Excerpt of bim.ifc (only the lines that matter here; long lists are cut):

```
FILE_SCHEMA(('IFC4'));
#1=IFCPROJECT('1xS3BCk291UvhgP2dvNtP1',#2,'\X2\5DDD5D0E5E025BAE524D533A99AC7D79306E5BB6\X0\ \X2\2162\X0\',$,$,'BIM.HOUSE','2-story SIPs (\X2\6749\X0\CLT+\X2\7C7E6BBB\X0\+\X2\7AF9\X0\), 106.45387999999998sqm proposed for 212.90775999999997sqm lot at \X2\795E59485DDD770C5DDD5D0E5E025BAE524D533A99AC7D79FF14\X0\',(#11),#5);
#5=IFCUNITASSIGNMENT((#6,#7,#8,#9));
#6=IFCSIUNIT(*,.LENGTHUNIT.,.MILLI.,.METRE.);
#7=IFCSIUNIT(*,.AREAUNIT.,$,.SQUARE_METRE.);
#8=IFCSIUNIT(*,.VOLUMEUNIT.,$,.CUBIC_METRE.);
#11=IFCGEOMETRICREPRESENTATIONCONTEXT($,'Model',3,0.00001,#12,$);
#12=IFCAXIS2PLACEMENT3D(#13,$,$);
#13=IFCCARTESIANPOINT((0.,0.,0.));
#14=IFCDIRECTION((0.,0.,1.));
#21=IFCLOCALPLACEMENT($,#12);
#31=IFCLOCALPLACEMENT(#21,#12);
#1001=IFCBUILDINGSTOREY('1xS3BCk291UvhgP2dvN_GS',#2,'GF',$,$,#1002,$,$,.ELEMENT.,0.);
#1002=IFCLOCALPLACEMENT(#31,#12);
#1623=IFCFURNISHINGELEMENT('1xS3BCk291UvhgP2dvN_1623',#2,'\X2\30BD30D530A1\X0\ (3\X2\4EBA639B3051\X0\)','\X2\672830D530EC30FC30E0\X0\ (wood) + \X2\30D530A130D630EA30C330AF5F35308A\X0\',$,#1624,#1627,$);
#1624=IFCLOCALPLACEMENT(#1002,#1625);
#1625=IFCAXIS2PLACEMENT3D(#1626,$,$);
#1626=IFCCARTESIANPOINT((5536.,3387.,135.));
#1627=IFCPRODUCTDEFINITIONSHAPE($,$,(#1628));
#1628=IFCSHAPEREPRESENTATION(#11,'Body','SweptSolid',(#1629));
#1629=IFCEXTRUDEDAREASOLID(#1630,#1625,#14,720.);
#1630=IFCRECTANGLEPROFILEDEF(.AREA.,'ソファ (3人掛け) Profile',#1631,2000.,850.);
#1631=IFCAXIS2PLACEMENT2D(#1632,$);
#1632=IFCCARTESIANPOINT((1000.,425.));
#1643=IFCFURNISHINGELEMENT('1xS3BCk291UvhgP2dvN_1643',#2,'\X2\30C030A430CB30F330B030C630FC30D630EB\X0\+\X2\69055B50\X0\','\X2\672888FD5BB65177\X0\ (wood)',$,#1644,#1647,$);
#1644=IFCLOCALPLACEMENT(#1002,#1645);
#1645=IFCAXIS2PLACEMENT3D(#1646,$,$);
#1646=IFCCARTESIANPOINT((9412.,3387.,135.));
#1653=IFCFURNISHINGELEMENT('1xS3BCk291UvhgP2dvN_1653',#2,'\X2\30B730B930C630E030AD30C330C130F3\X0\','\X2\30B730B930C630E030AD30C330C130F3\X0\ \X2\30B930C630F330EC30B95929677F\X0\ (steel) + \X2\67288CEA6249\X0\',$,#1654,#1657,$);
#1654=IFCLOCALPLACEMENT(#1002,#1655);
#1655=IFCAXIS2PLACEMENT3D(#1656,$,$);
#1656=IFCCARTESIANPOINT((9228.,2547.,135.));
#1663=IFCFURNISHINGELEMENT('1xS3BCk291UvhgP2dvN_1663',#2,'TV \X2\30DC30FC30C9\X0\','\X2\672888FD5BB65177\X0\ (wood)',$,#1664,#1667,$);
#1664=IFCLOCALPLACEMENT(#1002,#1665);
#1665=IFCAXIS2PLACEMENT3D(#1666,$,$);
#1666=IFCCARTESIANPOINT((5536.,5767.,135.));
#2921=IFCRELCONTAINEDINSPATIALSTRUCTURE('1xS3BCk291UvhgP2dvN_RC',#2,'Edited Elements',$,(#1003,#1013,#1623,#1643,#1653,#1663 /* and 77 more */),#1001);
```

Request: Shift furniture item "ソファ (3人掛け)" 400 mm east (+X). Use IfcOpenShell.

```python
import ifcopenshell
import ifcopenshell.api.geometry
import ifcopenshell.util.placement
import ifcopenshell.util.unit

model = ifcopenshell.open("bim.ifc")
unit_scale = ifcopenshell.util.unit.calculate_unit_scale(model)

item = model.by_guid("1xS3BCk291UvhgP2dvN_1623")
matrix = ifcopenshell.util.placement.get_local_placement(item.ObjectPlacement)
matrix[0, 3] += 0.4 / unit_scale
ifcopenshell.api.geometry.edit_object_placement(model, product=item, matrix=matrix, is_si=False)

print(ifcopenshell.util.placement.get_local_placement(item.ObjectPlacement).round(3) + 0.0)

model.write("bim-out.ifc")
```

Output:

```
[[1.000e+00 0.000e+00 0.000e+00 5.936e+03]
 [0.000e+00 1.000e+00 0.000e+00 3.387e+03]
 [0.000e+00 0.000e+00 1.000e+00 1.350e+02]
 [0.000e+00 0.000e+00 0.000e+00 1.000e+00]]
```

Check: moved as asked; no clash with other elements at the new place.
